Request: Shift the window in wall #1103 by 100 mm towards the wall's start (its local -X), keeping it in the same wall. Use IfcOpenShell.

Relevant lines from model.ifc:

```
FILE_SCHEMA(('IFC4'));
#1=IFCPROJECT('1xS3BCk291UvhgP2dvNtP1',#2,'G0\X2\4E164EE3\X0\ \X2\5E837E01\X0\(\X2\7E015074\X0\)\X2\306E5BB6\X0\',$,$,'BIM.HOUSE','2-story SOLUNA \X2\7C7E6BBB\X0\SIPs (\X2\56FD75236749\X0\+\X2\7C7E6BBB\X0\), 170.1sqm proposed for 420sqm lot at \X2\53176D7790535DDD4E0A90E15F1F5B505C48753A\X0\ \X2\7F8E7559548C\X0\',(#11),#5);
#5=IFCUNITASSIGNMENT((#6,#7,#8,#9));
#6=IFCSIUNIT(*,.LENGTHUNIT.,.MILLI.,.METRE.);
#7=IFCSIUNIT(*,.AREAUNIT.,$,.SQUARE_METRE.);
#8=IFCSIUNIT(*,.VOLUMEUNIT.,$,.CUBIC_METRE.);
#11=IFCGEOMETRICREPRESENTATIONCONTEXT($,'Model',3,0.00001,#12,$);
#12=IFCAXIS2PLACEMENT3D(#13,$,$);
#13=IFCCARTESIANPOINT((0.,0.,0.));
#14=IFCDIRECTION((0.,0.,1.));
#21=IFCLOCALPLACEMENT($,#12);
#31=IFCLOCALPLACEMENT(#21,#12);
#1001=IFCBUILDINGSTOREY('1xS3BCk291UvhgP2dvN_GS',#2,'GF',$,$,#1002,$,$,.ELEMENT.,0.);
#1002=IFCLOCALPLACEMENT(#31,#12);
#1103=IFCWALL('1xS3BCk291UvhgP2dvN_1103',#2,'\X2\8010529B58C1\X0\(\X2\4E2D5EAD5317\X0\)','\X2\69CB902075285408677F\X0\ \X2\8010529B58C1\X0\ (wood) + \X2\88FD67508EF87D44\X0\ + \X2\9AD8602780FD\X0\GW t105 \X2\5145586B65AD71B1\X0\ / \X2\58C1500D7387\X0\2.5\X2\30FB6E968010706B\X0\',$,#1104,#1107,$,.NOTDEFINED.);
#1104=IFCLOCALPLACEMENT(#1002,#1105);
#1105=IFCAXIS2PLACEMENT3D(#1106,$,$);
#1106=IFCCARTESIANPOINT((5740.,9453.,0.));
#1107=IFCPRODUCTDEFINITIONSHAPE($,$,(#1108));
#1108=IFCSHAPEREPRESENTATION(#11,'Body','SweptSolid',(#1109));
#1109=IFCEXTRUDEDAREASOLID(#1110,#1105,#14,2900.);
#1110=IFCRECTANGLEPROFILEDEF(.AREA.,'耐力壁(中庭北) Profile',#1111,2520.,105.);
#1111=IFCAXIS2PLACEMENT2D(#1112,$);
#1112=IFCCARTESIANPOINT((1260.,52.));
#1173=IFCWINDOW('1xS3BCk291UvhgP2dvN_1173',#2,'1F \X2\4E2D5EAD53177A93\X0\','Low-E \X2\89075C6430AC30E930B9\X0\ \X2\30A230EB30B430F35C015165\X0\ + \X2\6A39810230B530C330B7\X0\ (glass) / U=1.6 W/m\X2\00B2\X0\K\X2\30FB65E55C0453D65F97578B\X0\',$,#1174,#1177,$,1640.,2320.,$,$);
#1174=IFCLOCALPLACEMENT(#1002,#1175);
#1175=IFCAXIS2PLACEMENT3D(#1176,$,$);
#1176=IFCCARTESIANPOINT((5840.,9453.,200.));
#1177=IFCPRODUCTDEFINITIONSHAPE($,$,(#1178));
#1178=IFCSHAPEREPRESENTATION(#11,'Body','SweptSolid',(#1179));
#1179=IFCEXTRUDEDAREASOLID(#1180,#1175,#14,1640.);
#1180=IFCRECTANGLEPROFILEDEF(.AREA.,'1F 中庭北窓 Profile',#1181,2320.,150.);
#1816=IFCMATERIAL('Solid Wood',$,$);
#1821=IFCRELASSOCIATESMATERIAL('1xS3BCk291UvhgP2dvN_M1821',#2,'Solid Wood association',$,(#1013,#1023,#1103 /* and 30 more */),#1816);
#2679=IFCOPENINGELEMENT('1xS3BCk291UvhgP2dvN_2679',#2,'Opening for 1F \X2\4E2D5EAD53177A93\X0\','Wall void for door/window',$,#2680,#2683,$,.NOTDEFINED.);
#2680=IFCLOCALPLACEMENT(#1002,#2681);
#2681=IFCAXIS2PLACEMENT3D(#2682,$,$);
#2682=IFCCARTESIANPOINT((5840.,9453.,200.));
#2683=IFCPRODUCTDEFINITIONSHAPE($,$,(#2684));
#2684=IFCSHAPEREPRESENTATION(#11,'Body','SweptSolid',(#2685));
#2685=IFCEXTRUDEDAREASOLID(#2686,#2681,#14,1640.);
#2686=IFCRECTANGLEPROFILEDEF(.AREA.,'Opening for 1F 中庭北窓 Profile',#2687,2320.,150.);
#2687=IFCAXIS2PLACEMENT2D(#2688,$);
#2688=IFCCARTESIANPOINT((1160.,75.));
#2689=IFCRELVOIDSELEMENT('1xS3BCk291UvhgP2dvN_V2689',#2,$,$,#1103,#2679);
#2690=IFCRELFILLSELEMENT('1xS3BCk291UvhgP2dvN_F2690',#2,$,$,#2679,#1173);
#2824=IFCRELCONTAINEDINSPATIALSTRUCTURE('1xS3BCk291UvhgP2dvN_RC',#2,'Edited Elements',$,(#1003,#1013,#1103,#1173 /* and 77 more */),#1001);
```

```python
import ifcopenshell
import ifcopenshell.api.geometry
import ifcopenshell.util.placement
import ifcopenshell.util.unit

model = ifcopenshell.open("model.ifc")
unit_scale = ifcopenshell.util.unit.calculate_unit_scale(model)

window = model.by_id(1173)
opening = window.FillsVoids[0].RelatingOpeningElement
wall = opening.VoidsElements[0].RelatingBuildingElement

wall_matrix = ifcopenshell.util.placement.get_local_placement(wall.ObjectPlacement)
shift = wall_matrix[:3, 0] * -0.1 / unit_scale
before = ifcopenshell.util.placement.get_local_placement(window.ObjectPlacement)[:3, 3].copy()

# The window is not placed relative to its opening, so move both.
for product in (opening, window):
    matrix = ifcopenshell.util.placement.get_local_placement(product.ObjectPlacement)
    matrix[:3, 3] += shift
    ifcopenshell.api.geometry.edit_object_placement(model, product=product, matrix=matrix, is_si=False)

after = ifcopenshell.util.placement.get_local_placement(window.ObjectPlacement)[:3, 3]
print("window moved by", (after - before).round(3) + 0.0)

model.write("model_v2.ifc")
```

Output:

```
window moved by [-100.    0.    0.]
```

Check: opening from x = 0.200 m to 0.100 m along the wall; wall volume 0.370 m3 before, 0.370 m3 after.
